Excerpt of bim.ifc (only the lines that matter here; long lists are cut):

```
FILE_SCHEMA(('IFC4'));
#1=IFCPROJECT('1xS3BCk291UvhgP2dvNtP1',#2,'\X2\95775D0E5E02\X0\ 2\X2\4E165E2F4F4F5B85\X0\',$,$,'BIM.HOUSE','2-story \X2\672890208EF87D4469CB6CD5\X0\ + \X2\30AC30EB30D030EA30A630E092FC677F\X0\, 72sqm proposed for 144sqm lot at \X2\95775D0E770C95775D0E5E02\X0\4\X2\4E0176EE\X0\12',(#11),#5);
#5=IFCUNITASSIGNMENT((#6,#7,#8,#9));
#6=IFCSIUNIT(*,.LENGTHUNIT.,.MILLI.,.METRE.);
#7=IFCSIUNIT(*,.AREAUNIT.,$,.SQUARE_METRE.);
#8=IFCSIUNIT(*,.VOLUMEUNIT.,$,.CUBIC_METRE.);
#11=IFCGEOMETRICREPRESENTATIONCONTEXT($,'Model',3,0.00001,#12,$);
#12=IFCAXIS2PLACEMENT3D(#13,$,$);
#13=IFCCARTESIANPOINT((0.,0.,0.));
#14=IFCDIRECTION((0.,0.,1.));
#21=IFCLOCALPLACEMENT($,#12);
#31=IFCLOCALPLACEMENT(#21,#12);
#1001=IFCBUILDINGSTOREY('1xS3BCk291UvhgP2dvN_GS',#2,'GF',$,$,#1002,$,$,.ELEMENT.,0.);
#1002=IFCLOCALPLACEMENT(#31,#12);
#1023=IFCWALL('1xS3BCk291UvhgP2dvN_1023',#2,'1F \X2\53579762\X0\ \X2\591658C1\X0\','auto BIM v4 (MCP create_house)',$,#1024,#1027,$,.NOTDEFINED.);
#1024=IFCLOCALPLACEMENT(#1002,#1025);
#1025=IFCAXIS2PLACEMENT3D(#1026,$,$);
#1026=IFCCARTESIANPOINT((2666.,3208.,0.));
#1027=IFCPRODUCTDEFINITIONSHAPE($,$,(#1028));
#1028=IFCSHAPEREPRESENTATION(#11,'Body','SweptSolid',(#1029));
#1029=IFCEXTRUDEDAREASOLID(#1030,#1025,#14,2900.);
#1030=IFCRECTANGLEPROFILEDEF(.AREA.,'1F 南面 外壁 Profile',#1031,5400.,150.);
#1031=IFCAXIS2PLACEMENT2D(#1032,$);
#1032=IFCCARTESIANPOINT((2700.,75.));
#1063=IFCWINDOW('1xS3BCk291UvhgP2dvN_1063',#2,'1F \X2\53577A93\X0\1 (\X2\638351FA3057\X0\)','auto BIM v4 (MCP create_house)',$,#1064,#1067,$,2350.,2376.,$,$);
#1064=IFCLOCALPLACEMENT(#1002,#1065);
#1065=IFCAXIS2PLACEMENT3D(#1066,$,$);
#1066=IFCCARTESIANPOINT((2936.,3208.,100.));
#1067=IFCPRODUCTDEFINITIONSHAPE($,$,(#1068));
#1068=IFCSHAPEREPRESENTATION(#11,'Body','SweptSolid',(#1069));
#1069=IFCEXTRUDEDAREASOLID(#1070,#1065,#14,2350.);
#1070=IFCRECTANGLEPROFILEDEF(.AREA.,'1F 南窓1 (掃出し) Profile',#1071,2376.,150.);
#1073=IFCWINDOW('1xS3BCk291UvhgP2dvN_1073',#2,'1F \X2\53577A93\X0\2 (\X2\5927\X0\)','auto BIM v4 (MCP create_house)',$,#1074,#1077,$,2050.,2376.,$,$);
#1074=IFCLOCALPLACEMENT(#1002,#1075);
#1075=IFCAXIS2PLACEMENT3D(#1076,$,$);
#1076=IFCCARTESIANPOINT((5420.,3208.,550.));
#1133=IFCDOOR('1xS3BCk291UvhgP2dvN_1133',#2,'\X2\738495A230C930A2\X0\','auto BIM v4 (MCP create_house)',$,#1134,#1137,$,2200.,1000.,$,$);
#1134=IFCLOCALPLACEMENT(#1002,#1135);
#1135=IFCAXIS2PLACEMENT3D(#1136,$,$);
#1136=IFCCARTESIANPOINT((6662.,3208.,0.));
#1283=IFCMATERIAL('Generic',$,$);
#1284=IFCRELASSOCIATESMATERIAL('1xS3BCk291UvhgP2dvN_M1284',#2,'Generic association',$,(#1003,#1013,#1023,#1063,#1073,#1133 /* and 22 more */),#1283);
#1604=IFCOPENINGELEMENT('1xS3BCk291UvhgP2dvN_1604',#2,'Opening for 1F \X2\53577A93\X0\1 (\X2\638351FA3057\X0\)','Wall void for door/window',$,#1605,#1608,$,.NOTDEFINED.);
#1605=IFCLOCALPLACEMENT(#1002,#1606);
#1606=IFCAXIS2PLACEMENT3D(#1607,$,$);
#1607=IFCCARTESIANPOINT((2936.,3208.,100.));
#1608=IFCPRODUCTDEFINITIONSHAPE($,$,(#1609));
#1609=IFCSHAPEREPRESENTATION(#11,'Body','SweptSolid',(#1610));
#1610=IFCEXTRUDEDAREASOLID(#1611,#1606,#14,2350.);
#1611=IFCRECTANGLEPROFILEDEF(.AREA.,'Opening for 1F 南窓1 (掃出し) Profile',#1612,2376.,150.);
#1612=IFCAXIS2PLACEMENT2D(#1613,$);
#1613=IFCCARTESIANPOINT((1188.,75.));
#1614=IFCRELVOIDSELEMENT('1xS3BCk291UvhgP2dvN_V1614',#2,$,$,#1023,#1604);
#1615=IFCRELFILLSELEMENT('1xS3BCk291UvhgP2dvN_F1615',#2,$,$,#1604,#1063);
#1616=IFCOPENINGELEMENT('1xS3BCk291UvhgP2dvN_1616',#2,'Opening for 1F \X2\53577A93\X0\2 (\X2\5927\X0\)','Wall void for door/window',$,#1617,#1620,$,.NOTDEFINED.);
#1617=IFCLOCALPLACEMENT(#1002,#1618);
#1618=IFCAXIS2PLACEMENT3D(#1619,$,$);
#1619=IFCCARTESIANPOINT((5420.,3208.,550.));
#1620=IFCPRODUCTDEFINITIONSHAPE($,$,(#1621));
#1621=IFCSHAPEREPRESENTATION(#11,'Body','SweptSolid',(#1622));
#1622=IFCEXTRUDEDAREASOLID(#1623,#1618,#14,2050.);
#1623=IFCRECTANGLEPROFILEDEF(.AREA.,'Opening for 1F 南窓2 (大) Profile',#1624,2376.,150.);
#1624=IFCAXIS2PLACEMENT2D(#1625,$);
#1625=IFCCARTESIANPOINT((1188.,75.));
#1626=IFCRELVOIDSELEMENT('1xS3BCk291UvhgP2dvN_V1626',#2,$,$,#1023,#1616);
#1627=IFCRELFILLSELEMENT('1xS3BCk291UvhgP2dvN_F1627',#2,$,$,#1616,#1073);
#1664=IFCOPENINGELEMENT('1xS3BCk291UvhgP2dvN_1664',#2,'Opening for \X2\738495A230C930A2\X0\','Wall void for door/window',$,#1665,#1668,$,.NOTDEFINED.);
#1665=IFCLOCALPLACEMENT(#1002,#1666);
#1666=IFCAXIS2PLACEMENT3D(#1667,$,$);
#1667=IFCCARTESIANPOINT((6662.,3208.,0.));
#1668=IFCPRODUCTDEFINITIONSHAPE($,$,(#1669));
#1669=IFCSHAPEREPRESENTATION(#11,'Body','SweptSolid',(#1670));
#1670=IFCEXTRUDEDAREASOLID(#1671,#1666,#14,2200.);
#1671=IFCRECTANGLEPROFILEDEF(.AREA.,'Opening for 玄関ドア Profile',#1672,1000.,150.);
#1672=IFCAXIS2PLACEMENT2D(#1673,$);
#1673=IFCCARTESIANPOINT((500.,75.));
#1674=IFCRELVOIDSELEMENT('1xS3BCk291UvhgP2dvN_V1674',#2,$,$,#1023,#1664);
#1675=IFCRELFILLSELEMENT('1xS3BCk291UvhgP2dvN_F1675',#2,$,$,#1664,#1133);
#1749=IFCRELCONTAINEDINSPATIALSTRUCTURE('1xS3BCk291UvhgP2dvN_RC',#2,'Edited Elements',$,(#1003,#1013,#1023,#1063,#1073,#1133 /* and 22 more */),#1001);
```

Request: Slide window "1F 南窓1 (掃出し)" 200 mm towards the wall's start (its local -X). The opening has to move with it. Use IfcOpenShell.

```python
import ifcopenshell
import ifcopenshell.api.geometry
import ifcopenshell.util.placement
import ifcopenshell.util.unit

model = ifcopenshell.open("bim.ifc")
unit_scale = ifcopenshell.util.unit.calculate_unit_scale(model)

window = model.by_guid("1xS3BCk291UvhgP2dvN_1063")
opening = window.FillsVoids[0].RelatingOpeningElement
wall = opening.VoidsElements[0].RelatingBuildingElement

wall_matrix = ifcopenshell.util.placement.get_local_placement(wall.ObjectPlacement)
shift = wall_matrix[:3, 0] * -0.2 / unit_scale
before = ifcopenshell.util.placement.get_local_placement(window.ObjectPlacement)[:3, 3].copy()

# The window is not placed relative to its opening, so move both.
for product in (opening, window):
    matrix = ifcopenshell.util.placement.get_local_placement(product.ObjectPlacement)
    matrix[:3, 3] += shift
    ifcopenshell.api.geometry.edit_object_placement(model, product=product, matrix=matrix, is_si=False)

after = ifcopenshell.util.placement.get_local_placement(window.ObjectPlacement)[:3, 3]
print("window moved by", (after - before).round(3) + 0.0)

model.write("bim_updated.ifc")
```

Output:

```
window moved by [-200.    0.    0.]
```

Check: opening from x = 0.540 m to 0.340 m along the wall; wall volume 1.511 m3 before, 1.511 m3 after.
